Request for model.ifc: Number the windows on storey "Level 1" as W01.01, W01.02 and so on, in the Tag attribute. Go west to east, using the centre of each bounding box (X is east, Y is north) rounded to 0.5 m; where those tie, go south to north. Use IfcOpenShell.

First a look at what the model holds.

```python
import ifcopenshell
import ifcopenshell.util.element
import ifcopenshell.util.placement

model = ifcopenshell.open("model.ifc")
print(model.schema)
storey = next(s for s in model.by_type("IfcBuildingStorey") if s.Name == "Level 1")
windows = [e for e in ifcopenshell.util.element.get_decomposition(storey) if e.is_a("IfcWindow")]
for e in sorted(windows, key=lambda e: e.id()):
    origin = ifcopenshell.util.placement.get_local_placement(e.ObjectPlacement)[:3, 3]
    print(e.id(), e.Tag, e.Name, origin.round(2) + 0.0, sep=" | ")
```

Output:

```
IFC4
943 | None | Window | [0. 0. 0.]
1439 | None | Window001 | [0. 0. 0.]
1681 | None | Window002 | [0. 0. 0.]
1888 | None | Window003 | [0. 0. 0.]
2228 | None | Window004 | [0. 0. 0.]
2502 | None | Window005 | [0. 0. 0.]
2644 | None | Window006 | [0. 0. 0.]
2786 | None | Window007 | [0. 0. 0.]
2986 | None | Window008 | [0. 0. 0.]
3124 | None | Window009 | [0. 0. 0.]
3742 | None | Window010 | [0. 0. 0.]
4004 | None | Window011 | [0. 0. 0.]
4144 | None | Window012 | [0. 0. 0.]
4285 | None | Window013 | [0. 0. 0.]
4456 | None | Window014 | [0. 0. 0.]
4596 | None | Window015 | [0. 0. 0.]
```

```python
import ifcopenshell
import ifcopenshell.geom
import ifcopenshell.util.element
import ifcopenshell.util.shape

model = ifcopenshell.open("model.ifc")
settings = ifcopenshell.geom.settings()
settings.set("use-world-coords", True)


def centre(element):
    shape = ifcopenshell.geom.create_shape(settings, element)
    return ifcopenshell.util.shape.get_bbox_centroid(shape.geometry)


storey = next(s for s in model.by_type("IfcBuildingStorey") if s.Name == "Level 1")
windows = [e for e in ifcopenshell.util.element.get_decomposition(storey) if e.is_a("IfcWindow")]

# Insertion points can sit at a corner or the storey origin, so sort by the geometry (in metres).
centres = {e: centre(e) for e in windows}
windows.sort(key=lambda e: (round(centres[e][0] / 0.5), centres[e][1]))

for i, e in enumerate(windows, start=1):
    number = f"W01.{i:02d}"
    e.Tag = number
    print(e.id(), number)

model.write("model_updated.ifc")
```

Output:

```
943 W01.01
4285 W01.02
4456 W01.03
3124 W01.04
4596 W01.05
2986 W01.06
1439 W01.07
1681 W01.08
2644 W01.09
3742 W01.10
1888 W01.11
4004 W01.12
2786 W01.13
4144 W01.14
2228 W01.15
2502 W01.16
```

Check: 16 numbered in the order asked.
